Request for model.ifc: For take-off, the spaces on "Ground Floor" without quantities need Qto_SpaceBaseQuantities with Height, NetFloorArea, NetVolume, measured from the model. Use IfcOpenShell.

First a look at what the model holds.

```python
import ifcopenshell
import ifcopenshell.util.element
import ifcopenshell.util.unit

model = ifcopenshell.open("model.ifc")
print(model.schema)
for unit_type in ("LENGTHUNIT", "AREAUNIT", "VOLUMEUNIT"):
    print(unit_type, ifcopenshell.util.unit.calculate_unit_scale(model, unit_type))
storey = next(s for s in model.by_type("IfcBuildingStorey") if s.Name == "Ground Floor")
spaces = [e for e in ifcopenshell.util.element.get_decomposition(storey) if e.is_a("IfcSpace")]
for e in sorted(spaces, key=lambda e: e.id()):
    print(e.id(), e.is_a(), e.Name, list(ifcopenshell.util.element.get_psets(e, qtos_only=True)), sep=" | ")
```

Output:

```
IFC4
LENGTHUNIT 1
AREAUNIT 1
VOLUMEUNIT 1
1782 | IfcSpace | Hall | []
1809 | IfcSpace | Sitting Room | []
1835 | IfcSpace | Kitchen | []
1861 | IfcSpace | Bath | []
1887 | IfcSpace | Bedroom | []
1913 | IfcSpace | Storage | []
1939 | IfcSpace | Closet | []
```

```python
import ifcopenshell
import ifcopenshell.api.pset
import ifcopenshell.geom
import ifcopenshell.util.element
import ifcopenshell.util.shape
import ifcopenshell.util.unit

model = ifcopenshell.open("model.ifc")
unit_scale = ifcopenshell.util.unit.calculate_unit_scale(model)
area_scale = ifcopenshell.util.unit.calculate_unit_scale(model, "AREAUNIT")
volume_scale = ifcopenshell.util.unit.calculate_unit_scale(model, "VOLUMEUNIT")
settings = ifcopenshell.geom.settings()

storey = next(s for s in model.by_type("IfcBuildingStorey") if s.Name == "Ground Floor")
spaces = [e for e in ifcopenshell.util.element.get_decomposition(storey) if e.is_a("IfcSpace")]

for e in sorted(spaces, key=lambda e: e.id()):
    if ifcopenshell.util.element.get_psets(e, qtos_only=True, should_inherit=False):
        continue
    # Geometry comes back in metres, in the element's own axes.
    shape = ifcopenshell.geom.create_shape(settings, e)
    values = {
        "Height": ifcopenshell.util.shape.get_z(shape.geometry) / unit_scale,
        "NetFloorArea": ifcopenshell.util.shape.get_footprint_area(shape.geometry) / area_scale,
        "NetVolume": ifcopenshell.util.shape.get_volume(shape.geometry) / volume_scale,
    }
    qto = ifcopenshell.api.pset.add_qto(model, product=e, name="Qto_SpaceBaseQuantities")
    ifcopenshell.api.pset.edit_qto(model, qto=qto, properties=values)
    print(e.id(), {k: round(v, 3) for k, v in values.items()})

model.write("model_edited.ifc")
```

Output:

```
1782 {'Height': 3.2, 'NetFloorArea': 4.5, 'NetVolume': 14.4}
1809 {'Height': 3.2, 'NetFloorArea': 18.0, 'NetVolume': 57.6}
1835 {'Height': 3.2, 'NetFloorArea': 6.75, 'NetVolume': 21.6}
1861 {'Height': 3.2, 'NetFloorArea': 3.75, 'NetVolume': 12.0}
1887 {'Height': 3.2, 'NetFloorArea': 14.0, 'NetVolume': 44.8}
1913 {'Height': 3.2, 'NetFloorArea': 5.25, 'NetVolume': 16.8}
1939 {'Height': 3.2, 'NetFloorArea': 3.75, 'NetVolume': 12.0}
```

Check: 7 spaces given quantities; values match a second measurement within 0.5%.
